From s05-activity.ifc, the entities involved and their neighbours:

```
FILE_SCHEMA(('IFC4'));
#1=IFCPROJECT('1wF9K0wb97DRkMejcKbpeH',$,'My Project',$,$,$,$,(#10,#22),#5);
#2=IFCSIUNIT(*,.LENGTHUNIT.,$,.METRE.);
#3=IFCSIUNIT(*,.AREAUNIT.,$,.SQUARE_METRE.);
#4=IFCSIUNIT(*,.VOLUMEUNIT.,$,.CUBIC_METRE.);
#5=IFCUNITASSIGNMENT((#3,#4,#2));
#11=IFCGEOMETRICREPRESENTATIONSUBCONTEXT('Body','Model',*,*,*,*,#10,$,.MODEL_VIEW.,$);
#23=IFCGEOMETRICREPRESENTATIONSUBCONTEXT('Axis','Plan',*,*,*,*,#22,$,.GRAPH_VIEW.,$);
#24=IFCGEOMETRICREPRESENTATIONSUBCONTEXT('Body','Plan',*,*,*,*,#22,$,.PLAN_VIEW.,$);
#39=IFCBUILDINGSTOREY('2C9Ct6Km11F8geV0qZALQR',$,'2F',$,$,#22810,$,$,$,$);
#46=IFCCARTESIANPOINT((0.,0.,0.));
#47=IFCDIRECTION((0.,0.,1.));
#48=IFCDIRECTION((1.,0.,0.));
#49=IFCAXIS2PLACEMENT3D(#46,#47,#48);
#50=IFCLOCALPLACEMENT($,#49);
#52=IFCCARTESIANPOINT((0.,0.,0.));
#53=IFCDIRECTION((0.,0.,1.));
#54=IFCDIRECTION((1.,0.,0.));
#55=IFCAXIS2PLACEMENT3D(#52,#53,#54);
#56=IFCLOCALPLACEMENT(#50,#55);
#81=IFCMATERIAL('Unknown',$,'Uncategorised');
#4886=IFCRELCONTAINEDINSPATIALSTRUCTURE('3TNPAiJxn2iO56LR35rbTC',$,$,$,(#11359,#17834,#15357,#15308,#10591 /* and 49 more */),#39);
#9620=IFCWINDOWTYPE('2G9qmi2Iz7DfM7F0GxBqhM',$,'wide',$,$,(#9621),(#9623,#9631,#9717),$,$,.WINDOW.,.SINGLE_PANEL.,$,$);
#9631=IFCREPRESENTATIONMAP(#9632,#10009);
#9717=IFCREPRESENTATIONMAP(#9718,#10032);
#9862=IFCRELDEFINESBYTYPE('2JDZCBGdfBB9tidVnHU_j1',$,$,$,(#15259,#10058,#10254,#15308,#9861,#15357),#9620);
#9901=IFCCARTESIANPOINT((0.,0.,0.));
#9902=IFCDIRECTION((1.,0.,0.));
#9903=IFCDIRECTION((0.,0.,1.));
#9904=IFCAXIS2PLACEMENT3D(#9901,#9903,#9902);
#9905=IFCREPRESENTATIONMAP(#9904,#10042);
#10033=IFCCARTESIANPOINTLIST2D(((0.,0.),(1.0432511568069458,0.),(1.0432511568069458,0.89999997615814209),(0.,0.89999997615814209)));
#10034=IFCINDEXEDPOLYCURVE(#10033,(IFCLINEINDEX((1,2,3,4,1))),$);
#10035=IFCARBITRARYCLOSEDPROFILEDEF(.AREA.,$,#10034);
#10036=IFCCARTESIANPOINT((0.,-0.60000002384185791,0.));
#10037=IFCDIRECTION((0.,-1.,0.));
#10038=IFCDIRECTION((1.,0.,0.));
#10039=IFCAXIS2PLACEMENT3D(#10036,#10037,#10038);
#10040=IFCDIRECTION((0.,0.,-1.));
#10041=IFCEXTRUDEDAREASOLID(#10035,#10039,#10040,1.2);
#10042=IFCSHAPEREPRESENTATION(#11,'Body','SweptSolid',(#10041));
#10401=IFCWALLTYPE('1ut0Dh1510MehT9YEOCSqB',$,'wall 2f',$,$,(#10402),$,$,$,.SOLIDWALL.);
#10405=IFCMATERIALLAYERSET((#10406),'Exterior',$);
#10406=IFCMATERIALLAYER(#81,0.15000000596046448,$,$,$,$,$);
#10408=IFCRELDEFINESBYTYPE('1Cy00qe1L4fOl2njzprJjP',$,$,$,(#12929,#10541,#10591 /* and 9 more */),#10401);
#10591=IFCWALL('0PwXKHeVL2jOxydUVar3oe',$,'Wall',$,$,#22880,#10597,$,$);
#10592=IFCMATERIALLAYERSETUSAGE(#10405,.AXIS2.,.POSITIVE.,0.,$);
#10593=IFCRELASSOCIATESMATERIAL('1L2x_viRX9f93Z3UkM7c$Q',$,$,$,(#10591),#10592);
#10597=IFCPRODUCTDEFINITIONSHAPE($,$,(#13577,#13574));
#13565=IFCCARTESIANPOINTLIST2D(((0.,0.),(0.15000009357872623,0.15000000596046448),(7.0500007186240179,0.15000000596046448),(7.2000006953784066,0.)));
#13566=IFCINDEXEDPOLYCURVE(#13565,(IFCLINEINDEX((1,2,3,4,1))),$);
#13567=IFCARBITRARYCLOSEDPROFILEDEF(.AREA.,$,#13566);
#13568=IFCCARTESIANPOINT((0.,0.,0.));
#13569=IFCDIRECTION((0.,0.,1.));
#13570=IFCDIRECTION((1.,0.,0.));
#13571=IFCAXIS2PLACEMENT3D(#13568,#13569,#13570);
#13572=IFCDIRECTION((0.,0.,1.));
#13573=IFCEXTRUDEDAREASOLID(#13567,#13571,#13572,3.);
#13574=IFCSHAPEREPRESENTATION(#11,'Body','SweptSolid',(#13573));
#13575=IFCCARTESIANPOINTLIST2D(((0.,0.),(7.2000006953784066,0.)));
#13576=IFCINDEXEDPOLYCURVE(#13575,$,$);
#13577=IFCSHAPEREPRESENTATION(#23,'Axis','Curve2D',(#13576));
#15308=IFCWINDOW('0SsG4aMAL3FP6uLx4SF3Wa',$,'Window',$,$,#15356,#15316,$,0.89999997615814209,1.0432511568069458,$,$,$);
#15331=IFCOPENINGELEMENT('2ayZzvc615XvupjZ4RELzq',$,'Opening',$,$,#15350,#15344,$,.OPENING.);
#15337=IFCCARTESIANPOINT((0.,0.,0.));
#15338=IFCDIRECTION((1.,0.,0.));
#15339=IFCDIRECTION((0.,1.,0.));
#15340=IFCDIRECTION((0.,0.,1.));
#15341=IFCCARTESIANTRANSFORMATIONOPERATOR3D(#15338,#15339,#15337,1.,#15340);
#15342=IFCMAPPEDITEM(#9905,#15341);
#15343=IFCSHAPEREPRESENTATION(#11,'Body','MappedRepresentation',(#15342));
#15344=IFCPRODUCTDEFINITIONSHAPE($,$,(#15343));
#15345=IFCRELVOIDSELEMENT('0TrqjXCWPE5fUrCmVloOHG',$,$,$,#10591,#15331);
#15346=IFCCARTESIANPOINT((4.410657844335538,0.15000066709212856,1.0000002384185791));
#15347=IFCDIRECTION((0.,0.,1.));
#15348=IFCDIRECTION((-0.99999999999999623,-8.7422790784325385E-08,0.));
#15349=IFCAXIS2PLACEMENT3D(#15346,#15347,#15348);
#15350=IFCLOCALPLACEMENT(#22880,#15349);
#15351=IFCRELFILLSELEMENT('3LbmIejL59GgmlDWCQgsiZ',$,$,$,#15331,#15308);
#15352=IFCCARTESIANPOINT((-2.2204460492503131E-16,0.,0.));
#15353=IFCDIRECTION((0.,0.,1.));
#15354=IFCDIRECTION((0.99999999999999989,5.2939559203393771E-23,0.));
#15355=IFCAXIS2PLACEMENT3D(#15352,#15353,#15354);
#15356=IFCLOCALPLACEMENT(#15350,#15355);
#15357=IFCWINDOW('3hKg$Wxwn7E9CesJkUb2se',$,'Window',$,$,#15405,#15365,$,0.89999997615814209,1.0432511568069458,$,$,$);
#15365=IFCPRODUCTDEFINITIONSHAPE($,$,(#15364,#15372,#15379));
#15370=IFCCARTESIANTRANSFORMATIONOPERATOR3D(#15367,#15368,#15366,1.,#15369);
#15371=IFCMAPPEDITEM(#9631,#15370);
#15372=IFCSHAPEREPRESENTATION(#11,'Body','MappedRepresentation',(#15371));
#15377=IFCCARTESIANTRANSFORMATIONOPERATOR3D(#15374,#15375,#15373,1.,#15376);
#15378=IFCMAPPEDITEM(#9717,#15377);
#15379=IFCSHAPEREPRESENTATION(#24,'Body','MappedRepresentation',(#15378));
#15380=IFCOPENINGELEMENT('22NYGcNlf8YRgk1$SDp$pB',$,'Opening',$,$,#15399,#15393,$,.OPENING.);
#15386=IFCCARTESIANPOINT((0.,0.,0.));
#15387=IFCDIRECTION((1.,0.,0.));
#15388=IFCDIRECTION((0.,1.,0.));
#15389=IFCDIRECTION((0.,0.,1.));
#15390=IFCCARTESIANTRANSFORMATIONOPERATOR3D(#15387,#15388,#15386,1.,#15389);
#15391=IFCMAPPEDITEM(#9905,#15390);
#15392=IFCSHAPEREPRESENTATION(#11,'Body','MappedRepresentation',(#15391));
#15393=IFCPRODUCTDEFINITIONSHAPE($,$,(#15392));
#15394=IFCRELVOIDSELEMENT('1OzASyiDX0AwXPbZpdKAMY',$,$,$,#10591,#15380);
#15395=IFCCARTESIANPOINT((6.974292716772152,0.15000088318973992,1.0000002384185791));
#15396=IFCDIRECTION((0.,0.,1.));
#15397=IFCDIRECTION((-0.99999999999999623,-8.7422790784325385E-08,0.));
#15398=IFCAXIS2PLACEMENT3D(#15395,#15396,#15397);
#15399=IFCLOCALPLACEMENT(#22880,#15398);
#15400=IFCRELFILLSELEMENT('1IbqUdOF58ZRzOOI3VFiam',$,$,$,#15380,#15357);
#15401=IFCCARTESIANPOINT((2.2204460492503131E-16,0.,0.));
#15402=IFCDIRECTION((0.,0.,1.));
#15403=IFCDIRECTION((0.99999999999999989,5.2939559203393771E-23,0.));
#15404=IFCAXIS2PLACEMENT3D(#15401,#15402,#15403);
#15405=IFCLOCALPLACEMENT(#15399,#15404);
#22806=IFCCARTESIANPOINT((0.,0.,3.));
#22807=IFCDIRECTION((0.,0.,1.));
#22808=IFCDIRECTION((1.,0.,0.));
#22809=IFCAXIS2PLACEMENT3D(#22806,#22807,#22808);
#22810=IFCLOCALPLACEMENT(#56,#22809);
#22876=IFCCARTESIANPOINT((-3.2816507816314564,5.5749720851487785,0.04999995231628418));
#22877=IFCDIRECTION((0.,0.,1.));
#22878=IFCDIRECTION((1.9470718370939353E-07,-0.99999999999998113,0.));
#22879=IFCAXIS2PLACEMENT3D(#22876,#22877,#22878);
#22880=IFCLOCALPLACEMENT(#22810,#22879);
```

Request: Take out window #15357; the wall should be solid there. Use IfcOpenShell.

```python
import ifcopenshell
import ifcopenshell.api.feature
import ifcopenshell.api.root
import ifcopenshell.geom
import ifcopenshell.util.shape

model = ifcopenshell.open("s05-activity.ifc")
settings = ifcopenshell.geom.settings()


def volume(element):
    """Net volume in cubic metres, openings subtracted."""
    shape = ifcopenshell.geom.create_shape(settings, element)
    return ifcopenshell.util.shape.get_volume(shape.geometry)


window = model.by_guid("3hKg$Wxwn7E9CesJkUb2se")
opening = window.FillsVoids[0].RelatingOpeningElement
wall = opening.VoidsElements[0].RelatingBuildingElement
before = volume(wall)

ifcopenshell.api.root.remove_product(model, product=window)
ifcopenshell.api.feature.remove_feature(model, feature=opening)

after = volume(wall)

print(f"wall volume {before:.3f} -> {after:.3f} m3")

model.write("s05-activity_edited.ifc")
```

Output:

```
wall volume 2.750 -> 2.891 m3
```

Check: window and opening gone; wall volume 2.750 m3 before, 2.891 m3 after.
